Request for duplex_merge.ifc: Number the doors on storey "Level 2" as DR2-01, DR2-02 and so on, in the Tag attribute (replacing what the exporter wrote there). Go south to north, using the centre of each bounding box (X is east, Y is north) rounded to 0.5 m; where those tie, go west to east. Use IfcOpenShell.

First a look at what the model holds.

```python
import ifcopenshell
import ifcopenshell.util.element
import ifcopenshell.util.placement

model = ifcopenshell.open("duplex_merge.ifc")
print(model.schema)
storey = next(s for s in model.by_type("IfcBuildingStorey") if s.Name == "Level 2")
doors = [e for e in ifcopenshell.util.element.get_decomposition(storey) if e.is_a("IfcDoor")]
for e in sorted(doors, key=lambda e: e.id()):
    origin = ifcopenshell.util.placement.get_local_placement(e.ObjectPlacement)[:3, 3]
    print(e.id(), e.Tag, e.Name, origin.round(2) + 0.0, sep=" | ")
```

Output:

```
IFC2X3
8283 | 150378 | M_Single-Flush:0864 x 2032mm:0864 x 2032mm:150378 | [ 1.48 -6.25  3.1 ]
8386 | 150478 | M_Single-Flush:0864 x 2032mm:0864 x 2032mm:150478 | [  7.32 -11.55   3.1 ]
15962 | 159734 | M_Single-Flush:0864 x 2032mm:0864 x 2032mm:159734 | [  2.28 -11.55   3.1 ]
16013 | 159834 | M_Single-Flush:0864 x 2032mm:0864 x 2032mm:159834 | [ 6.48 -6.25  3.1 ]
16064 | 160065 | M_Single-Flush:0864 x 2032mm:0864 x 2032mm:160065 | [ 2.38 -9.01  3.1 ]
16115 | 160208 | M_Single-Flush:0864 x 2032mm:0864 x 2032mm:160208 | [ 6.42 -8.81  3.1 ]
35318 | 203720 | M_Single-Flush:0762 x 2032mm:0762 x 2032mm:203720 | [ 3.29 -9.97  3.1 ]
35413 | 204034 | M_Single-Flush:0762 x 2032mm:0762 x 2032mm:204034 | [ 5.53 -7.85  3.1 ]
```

```python
import ifcopenshell
import ifcopenshell.geom
import ifcopenshell.util.element
import ifcopenshell.util.shape

model = ifcopenshell.open("duplex_merge.ifc")
settings = ifcopenshell.geom.settings()
settings.set("use-world-coords", True)


def centre(element):
    shape = ifcopenshell.geom.create_shape(settings, element)
    return ifcopenshell.util.shape.get_bbox_centroid(shape.geometry)


storey = next(s for s in model.by_type("IfcBuildingStorey") if s.Name == "Level 2")
doors = [e for e in ifcopenshell.util.element.get_decomposition(storey) if e.is_a("IfcDoor")]

# Insertion points can sit at a corner or the storey origin, so sort by the geometry (in metres).
centres = {e: centre(e) for e in doors}
doors.sort(key=lambda e: (round(centres[e][1] / 0.5), centres[e][0]))

for i, e in enumerate(doors, start=1):
    number = f"DR2-{i:02d}"
    e.Tag = number
    print(e.id(), number)

model.write("duplex_merge_v2.ifc")
```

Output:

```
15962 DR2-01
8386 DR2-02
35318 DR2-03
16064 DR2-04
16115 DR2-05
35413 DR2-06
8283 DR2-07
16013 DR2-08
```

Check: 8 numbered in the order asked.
